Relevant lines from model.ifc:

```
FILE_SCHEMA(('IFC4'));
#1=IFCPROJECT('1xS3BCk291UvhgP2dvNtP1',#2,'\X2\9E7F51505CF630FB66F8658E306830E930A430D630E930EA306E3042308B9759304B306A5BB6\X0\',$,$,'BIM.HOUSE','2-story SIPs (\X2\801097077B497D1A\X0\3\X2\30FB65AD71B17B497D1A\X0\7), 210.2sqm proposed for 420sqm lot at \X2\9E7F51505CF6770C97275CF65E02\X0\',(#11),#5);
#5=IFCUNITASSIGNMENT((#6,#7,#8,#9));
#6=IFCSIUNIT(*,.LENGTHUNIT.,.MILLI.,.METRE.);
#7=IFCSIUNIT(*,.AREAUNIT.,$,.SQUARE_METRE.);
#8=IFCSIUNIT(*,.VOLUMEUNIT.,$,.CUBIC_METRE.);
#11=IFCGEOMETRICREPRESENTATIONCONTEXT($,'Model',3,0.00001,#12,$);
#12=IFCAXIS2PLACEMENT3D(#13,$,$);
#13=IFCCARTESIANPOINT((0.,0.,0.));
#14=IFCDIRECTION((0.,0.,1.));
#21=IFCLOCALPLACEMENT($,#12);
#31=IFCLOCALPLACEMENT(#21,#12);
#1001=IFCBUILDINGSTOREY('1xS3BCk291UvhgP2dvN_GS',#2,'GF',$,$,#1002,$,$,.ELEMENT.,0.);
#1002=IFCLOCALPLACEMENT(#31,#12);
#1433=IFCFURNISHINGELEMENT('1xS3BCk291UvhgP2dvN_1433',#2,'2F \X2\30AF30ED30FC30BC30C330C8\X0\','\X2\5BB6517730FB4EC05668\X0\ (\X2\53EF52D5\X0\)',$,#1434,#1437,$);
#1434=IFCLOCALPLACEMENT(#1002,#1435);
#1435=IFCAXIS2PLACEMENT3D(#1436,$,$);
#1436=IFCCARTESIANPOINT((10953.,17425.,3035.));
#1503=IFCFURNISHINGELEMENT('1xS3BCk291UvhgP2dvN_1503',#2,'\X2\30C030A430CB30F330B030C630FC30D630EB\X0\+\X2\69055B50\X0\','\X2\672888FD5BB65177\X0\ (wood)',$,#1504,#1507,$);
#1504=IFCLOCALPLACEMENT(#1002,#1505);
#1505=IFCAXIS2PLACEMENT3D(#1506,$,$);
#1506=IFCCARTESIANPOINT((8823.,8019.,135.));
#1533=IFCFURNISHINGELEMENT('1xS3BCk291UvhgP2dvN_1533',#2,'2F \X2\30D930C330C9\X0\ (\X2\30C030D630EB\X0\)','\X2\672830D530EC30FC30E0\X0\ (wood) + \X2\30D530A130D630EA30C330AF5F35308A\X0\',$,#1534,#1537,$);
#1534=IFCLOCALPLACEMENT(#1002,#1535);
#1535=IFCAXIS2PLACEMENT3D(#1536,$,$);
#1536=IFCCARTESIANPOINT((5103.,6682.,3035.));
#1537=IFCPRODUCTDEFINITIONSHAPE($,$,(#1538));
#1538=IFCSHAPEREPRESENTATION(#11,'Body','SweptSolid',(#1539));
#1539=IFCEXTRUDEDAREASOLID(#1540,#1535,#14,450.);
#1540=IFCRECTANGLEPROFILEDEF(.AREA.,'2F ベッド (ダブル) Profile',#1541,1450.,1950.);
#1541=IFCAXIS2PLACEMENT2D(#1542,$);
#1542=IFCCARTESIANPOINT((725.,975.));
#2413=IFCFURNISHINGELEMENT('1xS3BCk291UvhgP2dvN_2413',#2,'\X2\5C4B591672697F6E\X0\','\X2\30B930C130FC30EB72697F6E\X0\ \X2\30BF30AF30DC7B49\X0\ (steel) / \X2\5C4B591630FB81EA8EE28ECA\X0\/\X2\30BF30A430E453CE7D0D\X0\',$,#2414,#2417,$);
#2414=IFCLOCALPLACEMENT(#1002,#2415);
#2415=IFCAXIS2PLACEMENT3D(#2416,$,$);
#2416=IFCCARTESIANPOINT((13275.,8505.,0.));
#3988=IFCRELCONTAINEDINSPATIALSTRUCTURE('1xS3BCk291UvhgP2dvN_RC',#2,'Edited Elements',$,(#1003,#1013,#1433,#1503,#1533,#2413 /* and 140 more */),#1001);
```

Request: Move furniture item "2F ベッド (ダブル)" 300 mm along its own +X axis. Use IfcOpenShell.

```python
import ifcopenshell
import ifcopenshell.api.geometry
import ifcopenshell.util.placement
import ifcopenshell.util.unit

model = ifcopenshell.open("model.ifc")
unit_scale = ifcopenshell.util.unit.calculate_unit_scale(model)

item = model.by_guid("1xS3BCk291UvhgP2dvN_1533")
matrix = ifcopenshell.util.placement.get_local_placement(item.ObjectPlacement)
matrix[:3, 3] += matrix[:3, 0] * 0.3 / unit_scale
ifcopenshell.api.geometry.edit_object_placement(model, product=item, matrix=matrix, is_si=False)

print(ifcopenshell.util.placement.get_local_placement(item.ObjectPlacement).round(3) + 0.0)

model.write("model_rev.ifc")
```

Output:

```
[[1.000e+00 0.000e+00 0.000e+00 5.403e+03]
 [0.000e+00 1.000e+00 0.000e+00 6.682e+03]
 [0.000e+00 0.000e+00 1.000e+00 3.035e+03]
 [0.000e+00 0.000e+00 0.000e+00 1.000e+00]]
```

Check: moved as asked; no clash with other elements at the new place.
